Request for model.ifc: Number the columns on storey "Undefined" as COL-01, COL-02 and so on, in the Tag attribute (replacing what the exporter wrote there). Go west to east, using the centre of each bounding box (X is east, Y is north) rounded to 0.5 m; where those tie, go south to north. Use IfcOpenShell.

First a look at what the model holds.

```python
import ifcopenshell
import ifcopenshell.util.element
import ifcopenshell.util.placement

model = ifcopenshell.open("model.ifc")
print(model.schema)
storey = next(s for s in model.by_type("IfcBuildingStorey") if s.Name == "Undefined")
columns = [e for e in ifcopenshell.util.element.get_decomposition(storey) if e.is_a("IfcColumn")]
for e in sorted(columns, key=lambda e: e.id()):
    origin = ifcopenshell.util.placement.get_local_placement(e.ObjectPlacement)[:3, 3]
    print(e.id(), e.Tag, e.Name, origin.round(2) + 0.0, sep=" | ")
```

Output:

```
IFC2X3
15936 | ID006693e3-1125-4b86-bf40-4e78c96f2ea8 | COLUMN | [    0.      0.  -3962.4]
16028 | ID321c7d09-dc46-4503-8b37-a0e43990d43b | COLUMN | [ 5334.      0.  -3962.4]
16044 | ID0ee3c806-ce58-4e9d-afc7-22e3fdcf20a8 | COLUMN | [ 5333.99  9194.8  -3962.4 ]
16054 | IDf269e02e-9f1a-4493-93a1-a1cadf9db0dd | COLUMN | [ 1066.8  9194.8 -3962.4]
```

```python
import ifcopenshell
import ifcopenshell.geom
import ifcopenshell.util.element
import ifcopenshell.util.shape

model = ifcopenshell.open("model.ifc")
settings = ifcopenshell.geom.settings()
settings.set("use-world-coords", True)


def centre(element):
    shape = ifcopenshell.geom.create_shape(settings, element)
    return ifcopenshell.util.shape.get_bbox_centroid(shape.geometry)


storey = next(s for s in model.by_type("IfcBuildingStorey") if s.Name == "Undefined")
columns = [e for e in ifcopenshell.util.element.get_decomposition(storey) if e.is_a("IfcColumn")]

# Insertion points can sit at a corner or the storey origin, so sort by the geometry (in metres).
centres = {e: centre(e) for e in columns}
columns.sort(key=lambda e: (round(centres[e][0] / 0.5), centres[e][1]))

for i, e in enumerate(columns, start=1):
    number = f"COL-{i:02d}"
    e.Tag = number
    print(e.id(), number)

model.write("model-out.ifc")
```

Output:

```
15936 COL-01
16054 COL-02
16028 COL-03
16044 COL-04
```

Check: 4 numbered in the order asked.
